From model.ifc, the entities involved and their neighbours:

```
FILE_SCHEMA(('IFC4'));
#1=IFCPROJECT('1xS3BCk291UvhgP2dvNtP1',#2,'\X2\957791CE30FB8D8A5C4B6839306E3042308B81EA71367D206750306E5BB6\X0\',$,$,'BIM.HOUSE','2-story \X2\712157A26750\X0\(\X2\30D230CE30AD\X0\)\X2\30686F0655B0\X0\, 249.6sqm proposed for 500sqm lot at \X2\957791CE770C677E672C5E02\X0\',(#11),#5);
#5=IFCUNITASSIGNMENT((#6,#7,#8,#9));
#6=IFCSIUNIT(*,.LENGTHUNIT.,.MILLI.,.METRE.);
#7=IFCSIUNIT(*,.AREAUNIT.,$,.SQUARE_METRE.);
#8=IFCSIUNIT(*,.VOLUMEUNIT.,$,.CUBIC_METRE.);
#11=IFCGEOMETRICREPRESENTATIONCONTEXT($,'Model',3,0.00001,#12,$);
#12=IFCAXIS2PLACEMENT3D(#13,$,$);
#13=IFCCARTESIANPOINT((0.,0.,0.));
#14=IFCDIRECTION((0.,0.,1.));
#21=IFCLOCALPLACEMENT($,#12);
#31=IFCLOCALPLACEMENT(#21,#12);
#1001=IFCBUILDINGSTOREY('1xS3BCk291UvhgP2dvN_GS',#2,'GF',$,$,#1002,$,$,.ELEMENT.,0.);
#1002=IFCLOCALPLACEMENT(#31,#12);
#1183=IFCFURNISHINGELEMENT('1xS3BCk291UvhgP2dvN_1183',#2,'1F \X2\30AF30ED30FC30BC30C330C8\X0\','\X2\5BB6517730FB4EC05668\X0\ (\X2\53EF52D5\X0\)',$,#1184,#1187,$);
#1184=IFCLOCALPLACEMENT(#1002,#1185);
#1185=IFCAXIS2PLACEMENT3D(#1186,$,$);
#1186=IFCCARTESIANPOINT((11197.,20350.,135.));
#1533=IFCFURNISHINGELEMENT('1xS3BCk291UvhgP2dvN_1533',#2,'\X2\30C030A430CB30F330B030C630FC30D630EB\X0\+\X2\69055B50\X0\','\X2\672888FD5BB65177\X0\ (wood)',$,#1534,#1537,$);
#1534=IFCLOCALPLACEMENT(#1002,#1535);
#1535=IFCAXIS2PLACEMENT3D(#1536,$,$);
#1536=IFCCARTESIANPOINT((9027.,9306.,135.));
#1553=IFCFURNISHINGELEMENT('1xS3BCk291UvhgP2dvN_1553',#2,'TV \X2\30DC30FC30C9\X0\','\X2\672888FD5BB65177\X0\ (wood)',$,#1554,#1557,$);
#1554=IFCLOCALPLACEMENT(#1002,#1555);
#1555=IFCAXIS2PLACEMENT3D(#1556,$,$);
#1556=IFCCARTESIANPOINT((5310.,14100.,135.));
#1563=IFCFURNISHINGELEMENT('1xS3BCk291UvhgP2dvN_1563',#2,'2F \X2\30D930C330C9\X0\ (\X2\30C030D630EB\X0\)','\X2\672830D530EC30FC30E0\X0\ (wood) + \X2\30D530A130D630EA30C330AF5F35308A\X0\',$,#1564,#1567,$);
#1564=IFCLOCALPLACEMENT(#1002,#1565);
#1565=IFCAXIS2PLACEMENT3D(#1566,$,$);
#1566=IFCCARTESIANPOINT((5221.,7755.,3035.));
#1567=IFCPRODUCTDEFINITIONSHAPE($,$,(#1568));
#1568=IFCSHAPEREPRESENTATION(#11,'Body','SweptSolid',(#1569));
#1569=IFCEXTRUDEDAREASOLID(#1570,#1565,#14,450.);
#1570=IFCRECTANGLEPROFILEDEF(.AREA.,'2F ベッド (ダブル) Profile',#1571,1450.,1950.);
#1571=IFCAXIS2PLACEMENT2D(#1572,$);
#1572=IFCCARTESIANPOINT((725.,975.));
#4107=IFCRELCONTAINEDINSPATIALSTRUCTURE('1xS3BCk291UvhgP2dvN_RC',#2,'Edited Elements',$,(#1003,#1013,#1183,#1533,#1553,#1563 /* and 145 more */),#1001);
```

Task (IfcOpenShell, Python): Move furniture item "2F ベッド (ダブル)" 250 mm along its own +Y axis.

```python
import ifcopenshell
import ifcopenshell.api.geometry
import ifcopenshell.util.placement
import ifcopenshell.util.unit

model = ifcopenshell.open("model.ifc")
unit_scale = ifcopenshell.util.unit.calculate_unit_scale(model)

item = model.by_guid("1xS3BCk291UvhgP2dvN_1563")
matrix = ifcopenshell.util.placement.get_local_placement(item.ObjectPlacement)
matrix[:3, 3] += matrix[:3, 1] * 0.25 / unit_scale
ifcopenshell.api.geometry.edit_object_placement(model, product=item, matrix=matrix, is_si=False)

print(ifcopenshell.util.placement.get_local_placement(item.ObjectPlacement).round(3) + 0.0)

model.write("model_updated.ifc")
```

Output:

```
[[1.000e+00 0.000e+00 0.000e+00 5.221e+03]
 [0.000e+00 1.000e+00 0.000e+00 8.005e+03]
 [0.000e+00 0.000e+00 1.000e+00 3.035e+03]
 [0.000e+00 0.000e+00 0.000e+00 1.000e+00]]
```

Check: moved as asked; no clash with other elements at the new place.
